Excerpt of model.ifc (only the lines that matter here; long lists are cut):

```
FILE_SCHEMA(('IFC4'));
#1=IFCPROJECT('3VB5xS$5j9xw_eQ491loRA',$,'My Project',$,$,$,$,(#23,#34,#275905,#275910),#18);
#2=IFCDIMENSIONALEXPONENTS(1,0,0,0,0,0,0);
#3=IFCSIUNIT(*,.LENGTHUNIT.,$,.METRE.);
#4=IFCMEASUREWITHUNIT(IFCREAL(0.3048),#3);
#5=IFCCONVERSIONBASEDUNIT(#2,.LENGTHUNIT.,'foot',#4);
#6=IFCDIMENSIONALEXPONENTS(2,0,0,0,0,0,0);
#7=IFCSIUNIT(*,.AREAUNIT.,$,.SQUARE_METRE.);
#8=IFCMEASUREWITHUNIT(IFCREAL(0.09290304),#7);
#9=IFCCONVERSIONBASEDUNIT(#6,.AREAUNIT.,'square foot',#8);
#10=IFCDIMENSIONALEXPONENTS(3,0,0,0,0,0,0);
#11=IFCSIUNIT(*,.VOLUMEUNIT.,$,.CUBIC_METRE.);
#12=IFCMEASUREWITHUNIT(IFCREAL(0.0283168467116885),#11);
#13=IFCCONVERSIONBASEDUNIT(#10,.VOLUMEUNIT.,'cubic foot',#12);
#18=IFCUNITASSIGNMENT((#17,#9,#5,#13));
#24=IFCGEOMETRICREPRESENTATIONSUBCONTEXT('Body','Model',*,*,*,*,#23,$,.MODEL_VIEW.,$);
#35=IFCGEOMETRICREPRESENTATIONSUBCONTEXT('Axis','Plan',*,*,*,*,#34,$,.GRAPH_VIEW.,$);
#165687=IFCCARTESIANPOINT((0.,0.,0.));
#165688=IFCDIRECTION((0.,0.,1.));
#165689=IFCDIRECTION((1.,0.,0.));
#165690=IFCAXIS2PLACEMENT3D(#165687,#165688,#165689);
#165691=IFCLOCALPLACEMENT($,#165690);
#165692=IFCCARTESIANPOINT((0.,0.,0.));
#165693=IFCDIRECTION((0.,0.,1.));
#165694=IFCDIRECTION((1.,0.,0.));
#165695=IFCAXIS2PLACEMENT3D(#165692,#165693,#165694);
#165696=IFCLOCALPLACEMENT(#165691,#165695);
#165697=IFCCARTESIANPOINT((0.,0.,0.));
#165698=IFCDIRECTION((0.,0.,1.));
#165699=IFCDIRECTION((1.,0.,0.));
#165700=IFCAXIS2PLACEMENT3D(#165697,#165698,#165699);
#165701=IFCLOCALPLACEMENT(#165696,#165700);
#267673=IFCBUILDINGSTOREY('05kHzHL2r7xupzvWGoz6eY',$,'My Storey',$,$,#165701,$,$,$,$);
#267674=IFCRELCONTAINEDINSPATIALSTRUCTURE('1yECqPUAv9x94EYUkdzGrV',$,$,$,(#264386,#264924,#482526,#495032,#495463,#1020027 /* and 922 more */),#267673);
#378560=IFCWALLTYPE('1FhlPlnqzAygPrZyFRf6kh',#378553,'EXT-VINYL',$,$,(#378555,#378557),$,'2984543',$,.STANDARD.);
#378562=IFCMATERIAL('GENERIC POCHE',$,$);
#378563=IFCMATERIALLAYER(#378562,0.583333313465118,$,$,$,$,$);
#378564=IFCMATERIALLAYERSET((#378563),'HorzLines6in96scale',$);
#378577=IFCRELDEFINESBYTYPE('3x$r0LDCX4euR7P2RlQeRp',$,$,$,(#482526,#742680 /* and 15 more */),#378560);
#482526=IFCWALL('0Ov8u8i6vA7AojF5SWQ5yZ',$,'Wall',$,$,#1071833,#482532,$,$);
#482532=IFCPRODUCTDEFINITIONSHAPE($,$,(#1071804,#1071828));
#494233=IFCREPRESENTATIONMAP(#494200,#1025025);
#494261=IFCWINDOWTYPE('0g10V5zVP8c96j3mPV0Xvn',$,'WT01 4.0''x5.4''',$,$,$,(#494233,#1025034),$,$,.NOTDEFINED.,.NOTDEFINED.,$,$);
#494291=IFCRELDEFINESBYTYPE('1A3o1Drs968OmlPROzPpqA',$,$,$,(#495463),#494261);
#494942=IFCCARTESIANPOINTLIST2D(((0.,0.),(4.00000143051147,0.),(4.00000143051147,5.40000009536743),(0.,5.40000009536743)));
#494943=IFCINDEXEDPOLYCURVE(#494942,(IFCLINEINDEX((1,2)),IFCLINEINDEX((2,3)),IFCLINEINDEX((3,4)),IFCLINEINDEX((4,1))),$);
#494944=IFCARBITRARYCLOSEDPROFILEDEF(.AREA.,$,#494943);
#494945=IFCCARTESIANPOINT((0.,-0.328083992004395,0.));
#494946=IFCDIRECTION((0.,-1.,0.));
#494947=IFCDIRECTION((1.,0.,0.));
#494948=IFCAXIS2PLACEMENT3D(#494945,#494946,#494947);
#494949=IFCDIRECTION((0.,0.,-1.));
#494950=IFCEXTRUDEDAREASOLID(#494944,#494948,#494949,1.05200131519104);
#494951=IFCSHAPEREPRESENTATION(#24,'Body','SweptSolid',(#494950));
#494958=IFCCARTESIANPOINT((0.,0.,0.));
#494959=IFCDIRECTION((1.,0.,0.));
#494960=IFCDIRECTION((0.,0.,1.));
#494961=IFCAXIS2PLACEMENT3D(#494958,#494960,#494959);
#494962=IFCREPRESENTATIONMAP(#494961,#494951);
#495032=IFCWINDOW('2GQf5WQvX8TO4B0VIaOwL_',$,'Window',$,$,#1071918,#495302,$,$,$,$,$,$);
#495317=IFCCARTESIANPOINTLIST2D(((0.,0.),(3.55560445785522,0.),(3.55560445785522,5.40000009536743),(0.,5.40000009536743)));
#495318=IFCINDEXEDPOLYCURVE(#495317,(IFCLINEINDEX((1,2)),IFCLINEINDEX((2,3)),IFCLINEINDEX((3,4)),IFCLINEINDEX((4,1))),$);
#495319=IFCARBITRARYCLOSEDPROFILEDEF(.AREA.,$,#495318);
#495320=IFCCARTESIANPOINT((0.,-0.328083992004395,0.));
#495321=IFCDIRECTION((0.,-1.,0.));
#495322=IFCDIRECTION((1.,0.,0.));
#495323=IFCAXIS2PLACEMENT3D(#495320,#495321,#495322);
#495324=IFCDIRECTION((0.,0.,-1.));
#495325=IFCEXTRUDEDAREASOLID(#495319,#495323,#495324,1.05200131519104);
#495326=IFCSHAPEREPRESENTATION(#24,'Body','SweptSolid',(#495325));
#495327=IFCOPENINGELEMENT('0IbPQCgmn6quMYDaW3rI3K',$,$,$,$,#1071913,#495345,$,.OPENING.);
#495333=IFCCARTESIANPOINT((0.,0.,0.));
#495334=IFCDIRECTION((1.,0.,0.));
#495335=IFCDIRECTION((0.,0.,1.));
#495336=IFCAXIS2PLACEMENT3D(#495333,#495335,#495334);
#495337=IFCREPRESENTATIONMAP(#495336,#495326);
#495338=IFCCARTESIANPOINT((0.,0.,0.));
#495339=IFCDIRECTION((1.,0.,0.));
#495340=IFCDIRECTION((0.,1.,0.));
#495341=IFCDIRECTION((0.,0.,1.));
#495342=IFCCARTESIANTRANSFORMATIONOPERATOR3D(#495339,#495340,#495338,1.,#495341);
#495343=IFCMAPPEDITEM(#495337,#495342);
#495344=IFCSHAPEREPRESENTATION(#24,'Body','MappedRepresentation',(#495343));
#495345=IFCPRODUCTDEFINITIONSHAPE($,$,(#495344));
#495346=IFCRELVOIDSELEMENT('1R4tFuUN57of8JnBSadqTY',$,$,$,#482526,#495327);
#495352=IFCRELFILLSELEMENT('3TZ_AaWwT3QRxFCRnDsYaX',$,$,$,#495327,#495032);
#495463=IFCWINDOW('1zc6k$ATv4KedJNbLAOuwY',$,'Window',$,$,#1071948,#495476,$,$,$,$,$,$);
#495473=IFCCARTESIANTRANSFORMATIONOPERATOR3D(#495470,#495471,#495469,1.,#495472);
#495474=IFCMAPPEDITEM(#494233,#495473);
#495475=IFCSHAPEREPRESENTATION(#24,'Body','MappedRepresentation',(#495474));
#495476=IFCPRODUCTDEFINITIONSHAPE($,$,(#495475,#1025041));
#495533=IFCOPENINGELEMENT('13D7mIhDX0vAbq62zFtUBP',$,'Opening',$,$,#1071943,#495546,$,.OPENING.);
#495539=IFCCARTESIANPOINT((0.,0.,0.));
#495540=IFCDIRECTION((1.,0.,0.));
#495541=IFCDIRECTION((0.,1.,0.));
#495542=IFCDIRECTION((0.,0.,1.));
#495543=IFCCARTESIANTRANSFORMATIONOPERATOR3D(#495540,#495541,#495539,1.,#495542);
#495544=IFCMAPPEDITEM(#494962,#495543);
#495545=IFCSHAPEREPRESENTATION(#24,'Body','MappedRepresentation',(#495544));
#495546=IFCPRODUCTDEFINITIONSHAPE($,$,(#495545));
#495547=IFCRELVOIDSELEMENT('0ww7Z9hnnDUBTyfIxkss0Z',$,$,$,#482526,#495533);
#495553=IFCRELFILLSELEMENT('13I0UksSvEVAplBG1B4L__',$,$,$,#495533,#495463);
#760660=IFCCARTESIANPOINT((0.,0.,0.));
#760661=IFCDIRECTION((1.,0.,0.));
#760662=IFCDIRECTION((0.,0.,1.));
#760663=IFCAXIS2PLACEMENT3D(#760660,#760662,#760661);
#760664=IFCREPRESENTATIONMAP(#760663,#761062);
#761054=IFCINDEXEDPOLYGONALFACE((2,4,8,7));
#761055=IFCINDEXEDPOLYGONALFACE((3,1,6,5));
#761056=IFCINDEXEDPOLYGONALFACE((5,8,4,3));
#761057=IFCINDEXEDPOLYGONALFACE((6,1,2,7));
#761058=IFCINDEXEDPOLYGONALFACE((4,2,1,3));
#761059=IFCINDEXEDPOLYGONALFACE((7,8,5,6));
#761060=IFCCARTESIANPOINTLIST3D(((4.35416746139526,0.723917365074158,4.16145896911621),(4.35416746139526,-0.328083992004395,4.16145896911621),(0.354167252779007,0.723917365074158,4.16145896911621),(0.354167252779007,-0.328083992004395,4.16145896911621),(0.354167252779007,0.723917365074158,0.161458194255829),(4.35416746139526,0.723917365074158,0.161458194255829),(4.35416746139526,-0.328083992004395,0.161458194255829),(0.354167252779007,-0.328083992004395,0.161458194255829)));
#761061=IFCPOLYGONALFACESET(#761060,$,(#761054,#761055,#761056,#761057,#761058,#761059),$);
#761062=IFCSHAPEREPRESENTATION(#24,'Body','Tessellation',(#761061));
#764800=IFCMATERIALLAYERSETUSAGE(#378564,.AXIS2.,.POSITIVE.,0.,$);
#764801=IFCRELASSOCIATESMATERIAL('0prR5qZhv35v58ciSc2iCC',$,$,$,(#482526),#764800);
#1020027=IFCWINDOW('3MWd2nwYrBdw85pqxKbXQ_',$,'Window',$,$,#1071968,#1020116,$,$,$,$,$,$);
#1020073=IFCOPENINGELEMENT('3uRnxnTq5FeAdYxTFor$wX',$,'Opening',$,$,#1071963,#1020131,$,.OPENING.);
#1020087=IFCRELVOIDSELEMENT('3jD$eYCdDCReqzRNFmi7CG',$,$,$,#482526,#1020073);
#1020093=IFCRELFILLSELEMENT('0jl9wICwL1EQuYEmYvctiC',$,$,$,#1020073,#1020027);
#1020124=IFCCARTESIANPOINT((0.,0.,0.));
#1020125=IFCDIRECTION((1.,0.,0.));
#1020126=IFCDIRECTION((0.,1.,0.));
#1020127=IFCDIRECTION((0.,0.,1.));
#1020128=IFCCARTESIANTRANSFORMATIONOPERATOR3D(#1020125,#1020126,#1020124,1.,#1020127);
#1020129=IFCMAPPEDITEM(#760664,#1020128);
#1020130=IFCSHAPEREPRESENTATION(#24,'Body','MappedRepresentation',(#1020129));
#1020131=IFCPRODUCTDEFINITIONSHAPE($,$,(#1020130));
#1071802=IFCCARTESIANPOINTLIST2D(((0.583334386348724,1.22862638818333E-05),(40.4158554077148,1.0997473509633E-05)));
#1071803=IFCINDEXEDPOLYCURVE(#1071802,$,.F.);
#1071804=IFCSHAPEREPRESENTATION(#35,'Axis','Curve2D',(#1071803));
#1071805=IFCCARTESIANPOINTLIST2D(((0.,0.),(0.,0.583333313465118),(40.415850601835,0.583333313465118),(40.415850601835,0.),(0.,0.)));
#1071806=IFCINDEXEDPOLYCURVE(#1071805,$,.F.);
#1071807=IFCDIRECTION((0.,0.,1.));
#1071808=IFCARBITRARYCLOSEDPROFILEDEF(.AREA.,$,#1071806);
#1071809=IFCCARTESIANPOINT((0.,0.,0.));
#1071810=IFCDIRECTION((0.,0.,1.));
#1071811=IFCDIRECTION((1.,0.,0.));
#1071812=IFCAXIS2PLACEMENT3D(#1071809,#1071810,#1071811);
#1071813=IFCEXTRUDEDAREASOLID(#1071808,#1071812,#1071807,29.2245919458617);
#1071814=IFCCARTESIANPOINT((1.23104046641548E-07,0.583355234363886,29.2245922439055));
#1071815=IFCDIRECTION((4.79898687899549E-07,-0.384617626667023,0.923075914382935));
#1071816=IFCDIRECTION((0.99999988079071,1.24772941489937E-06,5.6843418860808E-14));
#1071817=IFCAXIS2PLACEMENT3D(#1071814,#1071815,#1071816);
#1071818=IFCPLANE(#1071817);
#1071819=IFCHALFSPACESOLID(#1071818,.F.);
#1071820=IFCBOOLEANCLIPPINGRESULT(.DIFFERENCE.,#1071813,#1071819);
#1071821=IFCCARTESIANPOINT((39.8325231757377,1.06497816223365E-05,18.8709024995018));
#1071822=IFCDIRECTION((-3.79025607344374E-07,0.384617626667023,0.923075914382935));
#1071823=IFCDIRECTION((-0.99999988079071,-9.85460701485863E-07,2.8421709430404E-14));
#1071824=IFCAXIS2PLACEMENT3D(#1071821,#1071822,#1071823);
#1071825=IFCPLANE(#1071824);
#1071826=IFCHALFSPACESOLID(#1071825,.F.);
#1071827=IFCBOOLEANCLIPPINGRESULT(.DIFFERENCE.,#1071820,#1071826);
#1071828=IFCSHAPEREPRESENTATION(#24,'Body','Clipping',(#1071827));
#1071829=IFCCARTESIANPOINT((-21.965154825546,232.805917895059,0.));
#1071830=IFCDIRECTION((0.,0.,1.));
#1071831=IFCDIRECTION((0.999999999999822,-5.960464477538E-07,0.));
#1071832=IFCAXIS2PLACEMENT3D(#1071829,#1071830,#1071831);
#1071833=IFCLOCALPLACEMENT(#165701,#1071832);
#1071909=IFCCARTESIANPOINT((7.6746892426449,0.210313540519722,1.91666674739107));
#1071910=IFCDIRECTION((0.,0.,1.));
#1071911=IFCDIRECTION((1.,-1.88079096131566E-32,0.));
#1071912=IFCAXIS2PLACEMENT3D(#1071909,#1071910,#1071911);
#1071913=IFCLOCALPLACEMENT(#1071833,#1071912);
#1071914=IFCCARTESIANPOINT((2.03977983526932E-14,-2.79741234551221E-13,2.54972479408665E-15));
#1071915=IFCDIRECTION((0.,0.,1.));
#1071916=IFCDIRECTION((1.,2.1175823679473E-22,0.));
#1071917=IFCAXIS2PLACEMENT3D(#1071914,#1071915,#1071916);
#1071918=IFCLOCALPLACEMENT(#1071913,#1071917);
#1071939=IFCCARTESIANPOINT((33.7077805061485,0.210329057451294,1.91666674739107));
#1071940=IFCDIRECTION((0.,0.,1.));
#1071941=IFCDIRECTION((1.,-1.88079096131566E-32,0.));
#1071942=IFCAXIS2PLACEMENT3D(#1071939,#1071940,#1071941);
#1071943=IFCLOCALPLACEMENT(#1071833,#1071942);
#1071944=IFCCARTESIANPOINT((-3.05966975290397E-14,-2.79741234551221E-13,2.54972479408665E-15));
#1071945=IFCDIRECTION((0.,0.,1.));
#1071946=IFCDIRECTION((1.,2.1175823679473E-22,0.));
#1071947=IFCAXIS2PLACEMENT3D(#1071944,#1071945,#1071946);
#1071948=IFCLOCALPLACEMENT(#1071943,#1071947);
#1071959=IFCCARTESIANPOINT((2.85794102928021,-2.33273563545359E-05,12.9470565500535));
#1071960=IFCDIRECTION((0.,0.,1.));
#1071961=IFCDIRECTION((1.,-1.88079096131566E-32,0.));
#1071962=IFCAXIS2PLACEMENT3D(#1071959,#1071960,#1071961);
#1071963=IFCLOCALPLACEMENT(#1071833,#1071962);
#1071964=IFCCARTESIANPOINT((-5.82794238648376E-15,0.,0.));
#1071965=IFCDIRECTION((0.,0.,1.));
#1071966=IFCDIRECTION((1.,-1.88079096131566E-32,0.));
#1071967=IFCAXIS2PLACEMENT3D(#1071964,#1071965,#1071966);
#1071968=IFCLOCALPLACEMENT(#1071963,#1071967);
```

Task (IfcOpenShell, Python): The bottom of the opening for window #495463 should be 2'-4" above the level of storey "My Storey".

```python
import numpy as np
import ifcopenshell
import ifcopenshell.api.geometry
import ifcopenshell.geom
import ifcopenshell.util.element
import ifcopenshell.util.placement
import ifcopenshell.util.shape
import ifcopenshell.util.unit

model = ifcopenshell.open("model.ifc")
unit_scale = ifcopenshell.util.unit.calculate_unit_scale(model)

window = model.by_guid("1zc6k$ATv4KedJNbLAOuwY")
opening = window.FillsVoids[0].RelatingOpeningElement
storey = ifcopenshell.util.element.get_container(window, ifc_class="IfcBuildingStorey")
level = ifcopenshell.util.placement.get_local_placement(storey.ObjectPlacement)[2, 3]

# The opening's origin need not be at the sill, so measure its lowest point.
shape = ifcopenshell.geom.create_shape(ifcopenshell.geom.settings(), opening)
bottom = ifcopenshell.util.shape.get_shape_bottom_elevation(shape, shape.geometry) / unit_scale
dz = level + 28 * 0.0254 / unit_scale - bottom

shift = np.array([0.0, 0.0, dz])
# The window is placed relative to its opening, so it follows when the opening moves.
matrix = ifcopenshell.util.placement.get_local_placement(opening.ObjectPlacement)
matrix[:3, 3] += shift
ifcopenshell.api.geometry.edit_object_placement(
    model, product=opening, matrix=matrix, is_si=False, should_transform_children=True
)

print(f"moved by {dz * unit_scale:+.3f} m")

model.write("model_rev.ifc")
```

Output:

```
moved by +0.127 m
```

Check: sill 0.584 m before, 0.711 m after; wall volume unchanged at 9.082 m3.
